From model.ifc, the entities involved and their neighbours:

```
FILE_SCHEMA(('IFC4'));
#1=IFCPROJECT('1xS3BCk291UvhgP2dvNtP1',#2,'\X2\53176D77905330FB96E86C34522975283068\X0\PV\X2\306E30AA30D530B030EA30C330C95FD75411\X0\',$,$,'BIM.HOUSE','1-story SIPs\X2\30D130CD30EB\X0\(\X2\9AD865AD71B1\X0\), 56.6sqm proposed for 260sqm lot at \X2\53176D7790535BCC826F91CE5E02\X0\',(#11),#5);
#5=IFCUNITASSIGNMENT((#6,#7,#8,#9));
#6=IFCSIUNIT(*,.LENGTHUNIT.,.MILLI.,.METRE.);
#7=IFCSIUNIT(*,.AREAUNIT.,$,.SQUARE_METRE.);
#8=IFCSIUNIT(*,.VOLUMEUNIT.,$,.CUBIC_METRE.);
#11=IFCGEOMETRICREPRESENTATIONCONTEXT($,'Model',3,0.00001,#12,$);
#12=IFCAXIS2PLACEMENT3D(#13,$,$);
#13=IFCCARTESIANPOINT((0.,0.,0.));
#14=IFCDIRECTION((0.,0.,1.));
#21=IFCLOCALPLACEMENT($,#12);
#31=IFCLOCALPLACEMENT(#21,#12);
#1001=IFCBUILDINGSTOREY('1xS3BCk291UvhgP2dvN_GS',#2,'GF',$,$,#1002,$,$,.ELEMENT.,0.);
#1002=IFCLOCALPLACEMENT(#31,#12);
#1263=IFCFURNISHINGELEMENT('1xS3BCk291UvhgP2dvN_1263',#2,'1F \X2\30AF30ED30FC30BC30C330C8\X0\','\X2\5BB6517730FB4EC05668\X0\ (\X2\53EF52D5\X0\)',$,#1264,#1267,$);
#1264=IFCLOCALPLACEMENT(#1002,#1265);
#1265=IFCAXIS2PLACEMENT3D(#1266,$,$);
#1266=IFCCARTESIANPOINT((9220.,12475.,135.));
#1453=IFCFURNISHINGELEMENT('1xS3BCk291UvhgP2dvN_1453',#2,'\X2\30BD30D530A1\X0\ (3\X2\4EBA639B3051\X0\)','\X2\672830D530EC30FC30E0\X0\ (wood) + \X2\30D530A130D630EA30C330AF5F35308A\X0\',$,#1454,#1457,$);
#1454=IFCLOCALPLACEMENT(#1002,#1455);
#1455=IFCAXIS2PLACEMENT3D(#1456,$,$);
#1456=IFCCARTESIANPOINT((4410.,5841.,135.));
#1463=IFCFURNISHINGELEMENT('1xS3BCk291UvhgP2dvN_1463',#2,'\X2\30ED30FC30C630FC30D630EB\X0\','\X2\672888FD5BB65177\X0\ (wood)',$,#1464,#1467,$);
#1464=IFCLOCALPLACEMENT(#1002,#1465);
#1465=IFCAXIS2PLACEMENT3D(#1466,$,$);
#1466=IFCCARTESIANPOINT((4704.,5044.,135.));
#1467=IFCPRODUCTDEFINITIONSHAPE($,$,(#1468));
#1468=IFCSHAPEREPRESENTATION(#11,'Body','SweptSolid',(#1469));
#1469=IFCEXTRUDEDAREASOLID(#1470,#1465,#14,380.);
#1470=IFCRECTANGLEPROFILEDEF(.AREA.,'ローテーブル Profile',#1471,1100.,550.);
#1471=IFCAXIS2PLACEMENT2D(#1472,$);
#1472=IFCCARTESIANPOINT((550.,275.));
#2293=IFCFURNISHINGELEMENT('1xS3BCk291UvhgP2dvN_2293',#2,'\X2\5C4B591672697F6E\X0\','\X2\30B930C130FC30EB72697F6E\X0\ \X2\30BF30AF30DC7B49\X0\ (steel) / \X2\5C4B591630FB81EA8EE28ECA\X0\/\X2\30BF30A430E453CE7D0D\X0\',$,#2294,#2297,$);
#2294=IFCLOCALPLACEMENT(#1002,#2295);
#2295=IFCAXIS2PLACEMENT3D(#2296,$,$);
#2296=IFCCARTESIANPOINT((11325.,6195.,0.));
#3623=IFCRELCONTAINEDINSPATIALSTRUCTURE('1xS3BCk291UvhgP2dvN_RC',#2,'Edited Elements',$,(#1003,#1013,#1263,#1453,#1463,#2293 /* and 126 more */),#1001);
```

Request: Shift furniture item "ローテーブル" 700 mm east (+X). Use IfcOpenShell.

```python
import ifcopenshell
import ifcopenshell.api.geometry
import ifcopenshell.util.placement

model = ifcopenshell.open("model.ifc")

item = model.by_id(1463)
matrix = ifcopenshell.util.placement.get_local_placement(item.ObjectPlacement)
matrix[0, 3] += 700.0
ifcopenshell.api.geometry.edit_object_placement(model, product=item, matrix=matrix, is_si=False)

print(ifcopenshell.util.placement.get_local_placement(item.ObjectPlacement).round(3) + 0.0)

model.write("model_edited.ifc")
```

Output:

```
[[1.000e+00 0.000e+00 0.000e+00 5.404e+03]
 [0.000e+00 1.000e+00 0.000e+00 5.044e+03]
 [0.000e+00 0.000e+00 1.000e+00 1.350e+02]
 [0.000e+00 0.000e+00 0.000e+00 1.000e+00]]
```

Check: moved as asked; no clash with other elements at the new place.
